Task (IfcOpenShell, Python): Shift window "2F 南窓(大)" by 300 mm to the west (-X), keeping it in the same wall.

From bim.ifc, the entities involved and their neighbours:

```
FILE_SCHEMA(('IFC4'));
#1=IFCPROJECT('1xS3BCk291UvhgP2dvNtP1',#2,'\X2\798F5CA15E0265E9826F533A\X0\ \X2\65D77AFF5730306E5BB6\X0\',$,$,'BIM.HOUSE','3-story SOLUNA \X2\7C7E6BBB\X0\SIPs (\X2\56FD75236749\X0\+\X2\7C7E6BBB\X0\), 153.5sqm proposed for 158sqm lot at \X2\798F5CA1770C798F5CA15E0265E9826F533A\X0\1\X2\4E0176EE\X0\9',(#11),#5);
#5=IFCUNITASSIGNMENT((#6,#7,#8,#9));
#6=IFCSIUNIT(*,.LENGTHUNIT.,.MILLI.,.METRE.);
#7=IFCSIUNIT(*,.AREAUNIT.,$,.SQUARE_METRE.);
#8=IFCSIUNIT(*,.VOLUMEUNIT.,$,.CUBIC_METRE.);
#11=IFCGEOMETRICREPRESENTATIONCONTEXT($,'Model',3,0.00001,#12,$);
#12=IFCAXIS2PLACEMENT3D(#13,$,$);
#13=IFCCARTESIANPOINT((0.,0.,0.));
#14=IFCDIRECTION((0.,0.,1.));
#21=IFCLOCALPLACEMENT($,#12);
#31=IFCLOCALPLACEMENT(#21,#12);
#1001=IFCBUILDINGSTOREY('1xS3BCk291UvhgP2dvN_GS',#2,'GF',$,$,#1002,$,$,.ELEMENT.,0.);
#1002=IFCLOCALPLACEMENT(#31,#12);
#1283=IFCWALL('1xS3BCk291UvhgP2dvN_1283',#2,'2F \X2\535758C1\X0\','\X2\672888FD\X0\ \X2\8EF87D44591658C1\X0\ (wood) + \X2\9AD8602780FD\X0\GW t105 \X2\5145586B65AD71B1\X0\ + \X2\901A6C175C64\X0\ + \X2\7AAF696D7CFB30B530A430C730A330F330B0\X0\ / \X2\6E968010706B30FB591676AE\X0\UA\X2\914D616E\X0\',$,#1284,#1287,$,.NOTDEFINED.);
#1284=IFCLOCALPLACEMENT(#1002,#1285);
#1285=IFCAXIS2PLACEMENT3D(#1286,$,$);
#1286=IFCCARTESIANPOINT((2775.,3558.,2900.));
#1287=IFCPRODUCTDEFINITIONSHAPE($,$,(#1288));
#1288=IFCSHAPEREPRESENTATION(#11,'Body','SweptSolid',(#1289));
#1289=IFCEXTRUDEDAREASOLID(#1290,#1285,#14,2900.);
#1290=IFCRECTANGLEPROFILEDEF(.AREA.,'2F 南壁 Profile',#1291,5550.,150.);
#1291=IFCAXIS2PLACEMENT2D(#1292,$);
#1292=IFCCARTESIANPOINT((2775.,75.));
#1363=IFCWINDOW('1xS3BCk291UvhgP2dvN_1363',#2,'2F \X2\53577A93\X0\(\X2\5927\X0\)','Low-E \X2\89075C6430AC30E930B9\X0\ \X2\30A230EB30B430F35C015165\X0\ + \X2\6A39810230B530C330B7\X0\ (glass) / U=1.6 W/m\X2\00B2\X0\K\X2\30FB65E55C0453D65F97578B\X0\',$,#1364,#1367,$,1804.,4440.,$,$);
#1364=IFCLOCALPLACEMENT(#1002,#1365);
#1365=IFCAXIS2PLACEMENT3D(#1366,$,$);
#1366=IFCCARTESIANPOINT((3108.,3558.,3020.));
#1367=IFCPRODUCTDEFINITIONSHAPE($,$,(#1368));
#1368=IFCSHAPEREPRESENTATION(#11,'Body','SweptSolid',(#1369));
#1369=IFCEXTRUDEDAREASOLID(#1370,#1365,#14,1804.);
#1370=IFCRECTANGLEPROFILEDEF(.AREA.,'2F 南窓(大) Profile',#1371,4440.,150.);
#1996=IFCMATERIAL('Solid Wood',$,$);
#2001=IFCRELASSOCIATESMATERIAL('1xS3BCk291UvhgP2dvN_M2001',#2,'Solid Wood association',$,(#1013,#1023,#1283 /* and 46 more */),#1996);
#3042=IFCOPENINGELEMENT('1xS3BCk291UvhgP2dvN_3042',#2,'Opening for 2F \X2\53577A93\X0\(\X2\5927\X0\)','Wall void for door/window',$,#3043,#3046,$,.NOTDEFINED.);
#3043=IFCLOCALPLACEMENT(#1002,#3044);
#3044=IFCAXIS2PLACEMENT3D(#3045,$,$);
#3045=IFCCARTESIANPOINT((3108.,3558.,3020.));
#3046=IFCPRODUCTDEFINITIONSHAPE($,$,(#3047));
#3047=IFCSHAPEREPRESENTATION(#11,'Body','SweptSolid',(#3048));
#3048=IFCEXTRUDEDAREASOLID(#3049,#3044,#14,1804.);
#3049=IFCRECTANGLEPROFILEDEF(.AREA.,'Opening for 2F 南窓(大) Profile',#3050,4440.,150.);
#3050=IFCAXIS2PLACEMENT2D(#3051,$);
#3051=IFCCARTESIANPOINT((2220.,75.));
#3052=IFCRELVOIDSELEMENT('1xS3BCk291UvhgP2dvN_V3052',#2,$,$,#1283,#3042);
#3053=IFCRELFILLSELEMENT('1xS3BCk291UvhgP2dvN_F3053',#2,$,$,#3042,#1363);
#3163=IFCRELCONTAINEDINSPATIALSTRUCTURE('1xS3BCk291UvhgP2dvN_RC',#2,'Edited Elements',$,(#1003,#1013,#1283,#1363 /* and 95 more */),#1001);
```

```python
import ifcopenshell
import ifcopenshell.api.geometry
import ifcopenshell.util.placement
import ifcopenshell.util.unit

model = ifcopenshell.open("bim.ifc")
unit_scale = ifcopenshell.util.unit.calculate_unit_scale(model)

window = model.by_guid("1xS3BCk291UvhgP2dvN_1363")
opening = window.FillsVoids[0].RelatingOpeningElement
wall = opening.VoidsElements[0].RelatingBuildingElement

wall_matrix = ifcopenshell.util.placement.get_local_placement(wall.ObjectPlacement)
shift = wall_matrix[:3, 0] * -0.3 / unit_scale
before = ifcopenshell.util.placement.get_local_placement(window.ObjectPlacement)[:3, 3].copy()

# The window is not placed relative to its opening, so move both.
for product in (opening, window):
    matrix = ifcopenshell.util.placement.get_local_placement(product.ObjectPlacement)
    matrix[:3, 3] += shift
    ifcopenshell.api.geometry.edit_object_placement(model, product=product, matrix=matrix, is_si=False)

after = ifcopenshell.util.placement.get_local_placement(window.ObjectPlacement)[:3, 3]
print("window moved by", (after - before).round(3) + 0.0)

model.write("bim_v2.ifc")
```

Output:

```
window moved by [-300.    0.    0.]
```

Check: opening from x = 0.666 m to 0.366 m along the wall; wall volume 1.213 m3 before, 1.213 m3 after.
